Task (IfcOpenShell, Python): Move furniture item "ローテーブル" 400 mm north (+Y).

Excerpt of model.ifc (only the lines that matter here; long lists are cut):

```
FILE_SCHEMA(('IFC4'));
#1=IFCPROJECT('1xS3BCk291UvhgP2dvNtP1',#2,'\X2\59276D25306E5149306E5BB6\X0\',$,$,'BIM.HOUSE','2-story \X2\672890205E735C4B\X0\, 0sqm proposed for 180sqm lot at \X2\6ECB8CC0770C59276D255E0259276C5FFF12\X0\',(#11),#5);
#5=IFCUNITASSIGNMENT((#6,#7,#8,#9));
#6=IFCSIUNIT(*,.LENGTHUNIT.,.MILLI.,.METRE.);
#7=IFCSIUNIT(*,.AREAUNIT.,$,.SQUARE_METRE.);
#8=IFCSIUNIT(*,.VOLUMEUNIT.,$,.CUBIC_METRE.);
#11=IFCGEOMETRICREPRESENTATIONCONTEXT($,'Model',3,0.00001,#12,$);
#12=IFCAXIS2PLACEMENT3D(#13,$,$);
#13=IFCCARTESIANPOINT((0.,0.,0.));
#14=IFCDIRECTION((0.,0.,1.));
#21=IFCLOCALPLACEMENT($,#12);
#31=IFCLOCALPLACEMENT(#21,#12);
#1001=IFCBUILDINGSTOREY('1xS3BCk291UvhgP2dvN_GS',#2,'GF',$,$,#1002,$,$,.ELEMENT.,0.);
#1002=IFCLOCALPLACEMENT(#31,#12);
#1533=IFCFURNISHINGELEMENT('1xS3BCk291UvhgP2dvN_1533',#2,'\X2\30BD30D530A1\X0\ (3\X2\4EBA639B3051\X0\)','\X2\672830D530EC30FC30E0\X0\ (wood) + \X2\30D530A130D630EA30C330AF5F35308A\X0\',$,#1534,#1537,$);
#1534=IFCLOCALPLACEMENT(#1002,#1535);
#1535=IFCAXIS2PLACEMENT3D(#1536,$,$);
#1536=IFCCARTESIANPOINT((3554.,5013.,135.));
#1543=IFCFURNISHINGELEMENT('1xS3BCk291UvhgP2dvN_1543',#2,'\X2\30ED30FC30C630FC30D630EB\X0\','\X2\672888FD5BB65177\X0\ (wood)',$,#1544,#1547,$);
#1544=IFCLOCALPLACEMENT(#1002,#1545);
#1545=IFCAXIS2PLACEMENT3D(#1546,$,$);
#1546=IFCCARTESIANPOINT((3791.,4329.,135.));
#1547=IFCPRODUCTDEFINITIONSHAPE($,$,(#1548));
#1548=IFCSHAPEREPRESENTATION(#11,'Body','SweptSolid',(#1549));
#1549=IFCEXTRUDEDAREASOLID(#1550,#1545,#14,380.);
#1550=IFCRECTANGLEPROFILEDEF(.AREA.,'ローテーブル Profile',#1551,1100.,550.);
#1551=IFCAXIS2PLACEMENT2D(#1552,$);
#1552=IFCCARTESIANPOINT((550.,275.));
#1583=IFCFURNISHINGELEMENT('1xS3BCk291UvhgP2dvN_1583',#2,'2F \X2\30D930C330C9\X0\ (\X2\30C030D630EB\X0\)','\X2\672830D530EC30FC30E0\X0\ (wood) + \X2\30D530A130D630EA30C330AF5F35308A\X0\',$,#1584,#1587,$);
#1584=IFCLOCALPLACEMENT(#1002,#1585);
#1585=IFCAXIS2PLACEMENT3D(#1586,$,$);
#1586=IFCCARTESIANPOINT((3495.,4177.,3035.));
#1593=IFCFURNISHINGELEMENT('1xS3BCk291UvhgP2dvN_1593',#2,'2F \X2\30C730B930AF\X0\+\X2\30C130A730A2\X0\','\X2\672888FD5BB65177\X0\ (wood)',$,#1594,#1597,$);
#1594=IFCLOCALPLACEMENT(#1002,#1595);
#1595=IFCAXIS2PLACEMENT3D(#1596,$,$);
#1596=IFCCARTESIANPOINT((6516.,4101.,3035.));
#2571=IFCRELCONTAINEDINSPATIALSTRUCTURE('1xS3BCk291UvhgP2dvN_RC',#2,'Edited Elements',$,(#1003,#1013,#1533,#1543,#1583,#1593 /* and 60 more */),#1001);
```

```python
import ifcopenshell
import ifcopenshell.api.geometry
import ifcopenshell.util.placement

model = ifcopenshell.open("model.ifc")

item = model.by_guid("1xS3BCk291UvhgP2dvN_1543")
matrix = ifcopenshell.util.placement.get_local_placement(item.ObjectPlacement)
matrix[1, 3] += 400.0
ifcopenshell.api.geometry.edit_object_placement(model, product=item, matrix=matrix, is_si=False)

print(ifcopenshell.util.placement.get_local_placement(item.ObjectPlacement).round(3) + 0.0)

model.write("model_edited.ifc")
```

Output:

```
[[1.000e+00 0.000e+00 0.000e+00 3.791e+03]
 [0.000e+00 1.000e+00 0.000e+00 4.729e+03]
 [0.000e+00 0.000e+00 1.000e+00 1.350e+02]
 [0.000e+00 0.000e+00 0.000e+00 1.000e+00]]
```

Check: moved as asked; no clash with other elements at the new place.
